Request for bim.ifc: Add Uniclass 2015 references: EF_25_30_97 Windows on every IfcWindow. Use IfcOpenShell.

First a look at what the model holds.

```python
import ifcopenshell

model = ifcopenshell.open("bim.ifc")
print(model.schema)
print("classifications:", [c.Name for c in model.by_type("IfcClassification")])
for ifc_class in ("IfcDoor", "IfcRoof", "IfcStair", "IfcWall", "IfcWindow"):
    print(ifc_class, len(model.by_type(ifc_class)))
```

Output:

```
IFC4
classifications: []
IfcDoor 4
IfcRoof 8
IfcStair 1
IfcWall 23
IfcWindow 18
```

```python
import ifcopenshell
import ifcopenshell.api.classification

model = ifcopenshell.open("bim.ifc")

system = ifcopenshell.api.classification.add_classification(model, classification="Uniclass 2015")

codes = {
    "IfcWindow": ("EF_25_30_97", "Windows"),
}
for ifc_class, (code, name) in codes.items():
    products = model.by_type(ifc_class)
    ifcopenshell.api.classification.add_reference(
        model, products=products, classification=system, identification=code, name=name
    )
    print(code, len(products))

model.write("bim_v2.ifc")
```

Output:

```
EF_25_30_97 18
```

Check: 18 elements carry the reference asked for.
